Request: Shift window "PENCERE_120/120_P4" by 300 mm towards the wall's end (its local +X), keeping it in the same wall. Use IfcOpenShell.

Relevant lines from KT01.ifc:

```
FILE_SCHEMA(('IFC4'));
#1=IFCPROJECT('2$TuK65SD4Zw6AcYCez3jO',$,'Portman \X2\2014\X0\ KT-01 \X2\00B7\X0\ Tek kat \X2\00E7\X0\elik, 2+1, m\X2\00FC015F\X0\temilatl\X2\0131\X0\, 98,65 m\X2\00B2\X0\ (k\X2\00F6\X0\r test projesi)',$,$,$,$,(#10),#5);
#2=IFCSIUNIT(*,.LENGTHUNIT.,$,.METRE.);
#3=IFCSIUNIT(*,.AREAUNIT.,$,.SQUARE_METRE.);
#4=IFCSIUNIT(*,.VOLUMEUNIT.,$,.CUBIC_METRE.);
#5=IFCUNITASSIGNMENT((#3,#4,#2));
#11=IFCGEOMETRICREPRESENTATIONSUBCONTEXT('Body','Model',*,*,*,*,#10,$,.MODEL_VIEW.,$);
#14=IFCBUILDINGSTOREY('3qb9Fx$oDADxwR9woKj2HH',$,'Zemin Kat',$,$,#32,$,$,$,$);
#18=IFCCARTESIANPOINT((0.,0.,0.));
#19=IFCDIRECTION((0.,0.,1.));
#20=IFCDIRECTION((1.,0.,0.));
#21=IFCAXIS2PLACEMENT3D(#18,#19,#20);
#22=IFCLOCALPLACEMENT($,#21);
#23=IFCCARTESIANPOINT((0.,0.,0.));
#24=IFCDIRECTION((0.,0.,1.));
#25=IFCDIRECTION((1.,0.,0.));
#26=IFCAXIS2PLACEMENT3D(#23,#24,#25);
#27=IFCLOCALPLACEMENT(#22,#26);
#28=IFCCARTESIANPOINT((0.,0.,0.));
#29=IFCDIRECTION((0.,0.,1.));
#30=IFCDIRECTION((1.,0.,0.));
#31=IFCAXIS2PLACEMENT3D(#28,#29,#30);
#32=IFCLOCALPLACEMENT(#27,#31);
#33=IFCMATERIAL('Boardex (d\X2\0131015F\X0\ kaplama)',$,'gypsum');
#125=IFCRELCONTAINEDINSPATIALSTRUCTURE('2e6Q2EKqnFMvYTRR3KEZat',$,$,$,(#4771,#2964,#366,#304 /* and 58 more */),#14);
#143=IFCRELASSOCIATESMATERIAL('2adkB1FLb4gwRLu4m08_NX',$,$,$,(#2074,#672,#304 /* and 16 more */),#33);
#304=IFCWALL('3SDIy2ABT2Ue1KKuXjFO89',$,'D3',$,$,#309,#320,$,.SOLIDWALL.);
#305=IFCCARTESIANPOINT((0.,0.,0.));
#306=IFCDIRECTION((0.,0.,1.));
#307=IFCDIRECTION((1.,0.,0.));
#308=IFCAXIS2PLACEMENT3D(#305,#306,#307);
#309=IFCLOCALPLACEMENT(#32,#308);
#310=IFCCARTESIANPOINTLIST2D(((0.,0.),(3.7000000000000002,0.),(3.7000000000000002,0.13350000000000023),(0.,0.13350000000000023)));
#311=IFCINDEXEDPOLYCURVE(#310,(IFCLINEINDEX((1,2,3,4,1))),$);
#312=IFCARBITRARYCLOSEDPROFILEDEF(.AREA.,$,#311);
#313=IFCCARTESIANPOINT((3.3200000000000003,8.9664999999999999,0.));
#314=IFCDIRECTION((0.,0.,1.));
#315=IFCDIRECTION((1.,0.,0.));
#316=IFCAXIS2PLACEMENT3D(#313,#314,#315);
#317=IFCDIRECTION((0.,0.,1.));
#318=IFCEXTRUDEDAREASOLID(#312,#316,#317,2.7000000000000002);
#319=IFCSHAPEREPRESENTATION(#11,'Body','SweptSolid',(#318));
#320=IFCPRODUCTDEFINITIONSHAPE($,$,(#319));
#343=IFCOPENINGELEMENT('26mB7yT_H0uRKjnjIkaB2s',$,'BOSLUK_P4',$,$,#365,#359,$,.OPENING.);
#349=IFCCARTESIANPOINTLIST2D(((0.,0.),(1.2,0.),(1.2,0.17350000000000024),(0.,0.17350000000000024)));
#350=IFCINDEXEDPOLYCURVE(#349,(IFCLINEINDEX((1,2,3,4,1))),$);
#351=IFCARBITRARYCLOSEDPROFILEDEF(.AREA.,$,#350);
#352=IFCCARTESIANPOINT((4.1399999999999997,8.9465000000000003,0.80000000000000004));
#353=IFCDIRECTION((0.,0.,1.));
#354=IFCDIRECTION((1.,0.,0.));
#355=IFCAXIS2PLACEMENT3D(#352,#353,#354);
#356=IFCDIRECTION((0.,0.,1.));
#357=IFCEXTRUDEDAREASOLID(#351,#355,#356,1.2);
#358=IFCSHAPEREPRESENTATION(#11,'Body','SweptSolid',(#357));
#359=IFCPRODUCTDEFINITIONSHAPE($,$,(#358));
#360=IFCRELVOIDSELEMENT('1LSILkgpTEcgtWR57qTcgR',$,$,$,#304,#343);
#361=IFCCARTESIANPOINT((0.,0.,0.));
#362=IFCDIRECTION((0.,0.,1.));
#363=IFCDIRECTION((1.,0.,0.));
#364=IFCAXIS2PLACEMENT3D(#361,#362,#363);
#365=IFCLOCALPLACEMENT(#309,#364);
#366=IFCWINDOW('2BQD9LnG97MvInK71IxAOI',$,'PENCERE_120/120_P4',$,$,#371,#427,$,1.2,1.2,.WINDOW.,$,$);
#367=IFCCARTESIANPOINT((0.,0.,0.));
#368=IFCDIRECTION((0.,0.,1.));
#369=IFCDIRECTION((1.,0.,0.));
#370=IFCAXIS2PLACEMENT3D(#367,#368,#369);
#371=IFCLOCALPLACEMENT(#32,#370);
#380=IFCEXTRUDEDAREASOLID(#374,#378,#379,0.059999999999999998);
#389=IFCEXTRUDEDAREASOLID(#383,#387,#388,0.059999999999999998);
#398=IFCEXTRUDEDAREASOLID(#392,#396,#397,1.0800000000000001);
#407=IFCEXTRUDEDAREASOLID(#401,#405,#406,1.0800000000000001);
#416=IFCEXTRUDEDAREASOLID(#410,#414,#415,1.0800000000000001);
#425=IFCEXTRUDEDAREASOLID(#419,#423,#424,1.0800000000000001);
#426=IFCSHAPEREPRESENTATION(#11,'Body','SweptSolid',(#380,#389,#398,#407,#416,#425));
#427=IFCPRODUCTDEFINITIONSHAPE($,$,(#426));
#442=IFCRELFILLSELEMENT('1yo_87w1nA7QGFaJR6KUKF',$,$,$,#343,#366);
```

```python
import ifcopenshell
import ifcopenshell.api.geometry
import ifcopenshell.util.placement
import ifcopenshell.util.unit

model = ifcopenshell.open("KT01.ifc")
unit_scale = ifcopenshell.util.unit.calculate_unit_scale(model)

window = model.by_guid("2BQD9LnG97MvInK71IxAOI")
opening = window.FillsVoids[0].RelatingOpeningElement
wall = opening.VoidsElements[0].RelatingBuildingElement

wall_matrix = ifcopenshell.util.placement.get_local_placement(wall.ObjectPlacement)
shift = wall_matrix[:3, 0] * 0.3 / unit_scale
before = ifcopenshell.util.placement.get_local_placement(window.ObjectPlacement)[:3, 3].copy()

# The window is not placed relative to its opening, so move both.
for product in (opening, window):
    matrix = ifcopenshell.util.placement.get_local_placement(product.ObjectPlacement)
    matrix[:3, 3] += shift
    ifcopenshell.api.geometry.edit_object_placement(model, product=product, matrix=matrix, is_si=False)

after = ifcopenshell.util.placement.get_local_placement(window.ObjectPlacement)[:3, 3]
print("window moved by", (after - before).round(3) + 0.0)

model.write("KT01_updated.ifc")
```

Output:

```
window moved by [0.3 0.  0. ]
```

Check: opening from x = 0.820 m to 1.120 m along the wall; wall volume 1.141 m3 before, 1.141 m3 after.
